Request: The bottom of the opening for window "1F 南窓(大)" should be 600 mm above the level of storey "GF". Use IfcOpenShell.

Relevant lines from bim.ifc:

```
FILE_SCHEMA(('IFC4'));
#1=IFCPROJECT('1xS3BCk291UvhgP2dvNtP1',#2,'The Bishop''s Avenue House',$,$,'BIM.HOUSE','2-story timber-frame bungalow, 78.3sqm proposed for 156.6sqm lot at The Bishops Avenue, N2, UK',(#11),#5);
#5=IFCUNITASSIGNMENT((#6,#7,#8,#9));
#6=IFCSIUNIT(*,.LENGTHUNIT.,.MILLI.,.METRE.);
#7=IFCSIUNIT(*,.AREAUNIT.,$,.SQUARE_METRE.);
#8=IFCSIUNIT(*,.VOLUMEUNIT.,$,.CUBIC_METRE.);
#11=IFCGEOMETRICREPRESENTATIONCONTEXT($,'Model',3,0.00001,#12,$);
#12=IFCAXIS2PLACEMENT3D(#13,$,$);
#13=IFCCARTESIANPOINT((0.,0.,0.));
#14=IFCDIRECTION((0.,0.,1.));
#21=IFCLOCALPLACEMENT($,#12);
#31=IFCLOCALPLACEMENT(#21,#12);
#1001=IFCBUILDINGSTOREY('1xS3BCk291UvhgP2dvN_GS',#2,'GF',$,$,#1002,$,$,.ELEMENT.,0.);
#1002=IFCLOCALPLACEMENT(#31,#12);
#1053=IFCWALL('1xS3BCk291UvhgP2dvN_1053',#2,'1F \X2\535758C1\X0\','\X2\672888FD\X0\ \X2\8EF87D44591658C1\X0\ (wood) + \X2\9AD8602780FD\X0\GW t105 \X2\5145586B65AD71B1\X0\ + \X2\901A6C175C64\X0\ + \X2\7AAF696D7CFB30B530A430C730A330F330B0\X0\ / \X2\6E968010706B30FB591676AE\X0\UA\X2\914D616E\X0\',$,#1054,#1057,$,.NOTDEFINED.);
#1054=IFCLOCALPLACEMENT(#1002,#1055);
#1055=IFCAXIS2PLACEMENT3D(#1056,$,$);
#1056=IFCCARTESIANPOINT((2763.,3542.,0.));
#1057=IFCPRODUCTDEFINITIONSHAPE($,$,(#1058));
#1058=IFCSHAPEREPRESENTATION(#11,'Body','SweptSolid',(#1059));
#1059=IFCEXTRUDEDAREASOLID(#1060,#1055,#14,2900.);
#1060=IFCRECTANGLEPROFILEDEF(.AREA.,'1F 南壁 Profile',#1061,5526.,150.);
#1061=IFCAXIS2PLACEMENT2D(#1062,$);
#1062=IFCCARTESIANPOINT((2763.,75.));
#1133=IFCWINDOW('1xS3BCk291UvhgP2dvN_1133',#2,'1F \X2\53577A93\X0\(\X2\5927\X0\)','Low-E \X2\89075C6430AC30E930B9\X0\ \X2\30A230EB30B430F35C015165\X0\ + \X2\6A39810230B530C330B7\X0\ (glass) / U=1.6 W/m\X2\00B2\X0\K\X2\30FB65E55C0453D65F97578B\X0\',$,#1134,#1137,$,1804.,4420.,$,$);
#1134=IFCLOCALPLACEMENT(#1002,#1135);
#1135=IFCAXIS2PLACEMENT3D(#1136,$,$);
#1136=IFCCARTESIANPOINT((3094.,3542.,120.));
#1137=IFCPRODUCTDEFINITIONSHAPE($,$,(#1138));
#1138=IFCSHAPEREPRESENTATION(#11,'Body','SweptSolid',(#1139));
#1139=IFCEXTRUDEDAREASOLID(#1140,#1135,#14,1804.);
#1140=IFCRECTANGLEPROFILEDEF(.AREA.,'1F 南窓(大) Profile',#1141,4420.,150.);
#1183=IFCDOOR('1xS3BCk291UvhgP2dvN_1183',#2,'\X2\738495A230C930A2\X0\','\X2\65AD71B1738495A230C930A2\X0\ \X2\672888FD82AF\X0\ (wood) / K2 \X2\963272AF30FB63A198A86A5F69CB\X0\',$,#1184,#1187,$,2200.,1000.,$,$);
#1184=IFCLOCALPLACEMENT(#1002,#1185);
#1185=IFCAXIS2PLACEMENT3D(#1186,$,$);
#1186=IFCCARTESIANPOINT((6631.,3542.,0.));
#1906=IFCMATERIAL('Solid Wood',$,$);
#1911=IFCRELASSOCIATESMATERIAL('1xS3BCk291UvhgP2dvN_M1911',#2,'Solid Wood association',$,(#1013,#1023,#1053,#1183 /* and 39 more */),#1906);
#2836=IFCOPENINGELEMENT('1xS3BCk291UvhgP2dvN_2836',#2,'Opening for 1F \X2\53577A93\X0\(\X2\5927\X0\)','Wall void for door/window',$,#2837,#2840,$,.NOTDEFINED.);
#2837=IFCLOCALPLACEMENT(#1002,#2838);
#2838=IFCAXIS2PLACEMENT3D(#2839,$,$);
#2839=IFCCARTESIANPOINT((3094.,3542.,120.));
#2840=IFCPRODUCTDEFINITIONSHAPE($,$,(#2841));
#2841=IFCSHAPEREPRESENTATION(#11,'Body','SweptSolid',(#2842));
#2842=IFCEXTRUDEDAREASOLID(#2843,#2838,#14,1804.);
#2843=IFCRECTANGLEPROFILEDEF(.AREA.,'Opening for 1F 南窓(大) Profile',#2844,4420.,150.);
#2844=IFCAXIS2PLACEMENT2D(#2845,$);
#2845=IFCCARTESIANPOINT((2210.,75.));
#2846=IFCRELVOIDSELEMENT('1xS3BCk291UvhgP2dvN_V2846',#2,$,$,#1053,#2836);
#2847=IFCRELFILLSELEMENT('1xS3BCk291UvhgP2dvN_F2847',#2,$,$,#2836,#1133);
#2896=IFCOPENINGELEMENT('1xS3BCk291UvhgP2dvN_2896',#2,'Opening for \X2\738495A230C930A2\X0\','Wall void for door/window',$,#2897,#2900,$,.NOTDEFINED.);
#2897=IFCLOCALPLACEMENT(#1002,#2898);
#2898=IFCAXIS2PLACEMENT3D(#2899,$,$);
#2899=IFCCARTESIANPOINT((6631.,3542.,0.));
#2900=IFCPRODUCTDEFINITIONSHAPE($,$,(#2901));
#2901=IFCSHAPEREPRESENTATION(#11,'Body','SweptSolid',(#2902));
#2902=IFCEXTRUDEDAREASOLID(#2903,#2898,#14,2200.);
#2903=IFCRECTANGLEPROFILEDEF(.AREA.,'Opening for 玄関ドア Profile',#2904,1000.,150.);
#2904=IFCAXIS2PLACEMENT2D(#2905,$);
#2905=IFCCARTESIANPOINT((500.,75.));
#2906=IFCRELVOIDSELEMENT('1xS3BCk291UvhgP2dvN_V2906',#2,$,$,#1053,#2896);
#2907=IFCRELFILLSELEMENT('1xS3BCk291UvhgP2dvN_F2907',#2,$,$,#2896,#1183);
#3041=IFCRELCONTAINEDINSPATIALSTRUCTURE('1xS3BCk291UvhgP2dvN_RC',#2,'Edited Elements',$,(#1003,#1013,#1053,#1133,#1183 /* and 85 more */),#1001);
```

```python
import numpy as np
import ifcopenshell
import ifcopenshell.api.geometry
import ifcopenshell.geom
import ifcopenshell.util.element
import ifcopenshell.util.placement
import ifcopenshell.util.shape
import ifcopenshell.util.unit

model = ifcopenshell.open("bim.ifc")
unit_scale = ifcopenshell.util.unit.calculate_unit_scale(model)

window = model.by_id(1133)
opening = window.FillsVoids[0].RelatingOpeningElement
storey = ifcopenshell.util.element.get_container(window, ifc_class="IfcBuildingStorey")
level = ifcopenshell.util.placement.get_local_placement(storey.ObjectPlacement)[2, 3]

# The opening's origin need not be at the sill, so measure its lowest point.
shape = ifcopenshell.geom.create_shape(ifcopenshell.geom.settings(), opening)
bottom = ifcopenshell.util.shape.get_shape_bottom_elevation(shape, shape.geometry) / unit_scale
dz = level + 600.0 - bottom

shift = np.array([0.0, 0.0, dz])
# The window is not placed relative to its opening, so move both.
for product in (opening, window):
    matrix = ifcopenshell.util.placement.get_local_placement(product.ObjectPlacement)
    matrix[:3, 3] += shift
    ifcopenshell.api.geometry.edit_object_placement(model, product=product, matrix=matrix, is_si=False)

print(f"moved by {dz * unit_scale:+.3f} m")

model.write("bim_v2.ifc")
```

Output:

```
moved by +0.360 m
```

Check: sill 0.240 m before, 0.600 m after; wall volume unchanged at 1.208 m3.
